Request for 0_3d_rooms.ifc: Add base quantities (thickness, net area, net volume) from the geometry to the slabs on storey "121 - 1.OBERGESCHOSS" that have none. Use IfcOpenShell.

First a look at what the model holds.

```python
import ifcopenshell
import ifcopenshell.util.element
import ifcopenshell.util.unit

model = ifcopenshell.open("0_3d_rooms.ifc")
print(model.schema)
for unit_type in ("LENGTHUNIT", "AREAUNIT", "VOLUMEUNIT"):
    print(unit_type, ifcopenshell.util.unit.calculate_unit_scale(model, unit_type))
storey = next(s for s in model.by_type("IfcBuildingStorey") if s.Name == "121 - 1.OBERGESCHOSS")
slabs = [e for e in ifcopenshell.util.element.get_decomposition(storey) if e.is_a("IfcSlab")]
for e in sorted(slabs, key=lambda e: e.id()):
    print(e.id(), e.is_a(), e.Name, list(ifcopenshell.util.element.get_psets(e, qtos_only=True)), sep=" | ")
```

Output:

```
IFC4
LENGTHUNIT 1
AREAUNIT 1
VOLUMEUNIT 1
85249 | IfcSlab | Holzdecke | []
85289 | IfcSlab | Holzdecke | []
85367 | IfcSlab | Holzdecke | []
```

```python
import ifcopenshell
import ifcopenshell.api.pset
import ifcopenshell.geom
import ifcopenshell.util.element
import ifcopenshell.util.shape
import ifcopenshell.util.unit

model = ifcopenshell.open("0_3d_rooms.ifc")
unit_scale = ifcopenshell.util.unit.calculate_unit_scale(model)
area_scale = ifcopenshell.util.unit.calculate_unit_scale(model, "AREAUNIT")
volume_scale = ifcopenshell.util.unit.calculate_unit_scale(model, "VOLUMEUNIT")
settings = ifcopenshell.geom.settings()

storey = next(s for s in model.by_type("IfcBuildingStorey") if s.Name == "121 - 1.OBERGESCHOSS")
slabs = [e for e in ifcopenshell.util.element.get_decomposition(storey) if e.is_a("IfcSlab")]

for e in sorted(slabs, key=lambda e: e.id()):
    if ifcopenshell.util.element.get_psets(e, qtos_only=True, should_inherit=False):
        continue
    # Geometry comes back in metres, in the element's own axes.
    shape = ifcopenshell.geom.create_shape(settings, e)
    values = {
        "Width": ifcopenshell.util.shape.get_z(shape.geometry) / unit_scale,
        "NetArea": ifcopenshell.util.shape.get_footprint_area(shape.geometry) / area_scale,
        "NetVolume": ifcopenshell.util.shape.get_volume(shape.geometry) / volume_scale,
    }
    qto = ifcopenshell.api.pset.add_qto(model, product=e, name="Qto_SlabBaseQuantities")
    ifcopenshell.api.pset.edit_qto(model, qto=qto, properties=values)
    print(e.id(), {k: round(v, 3) for k, v in values.items()})

model.write("0_3d_rooms-out.ifc")
```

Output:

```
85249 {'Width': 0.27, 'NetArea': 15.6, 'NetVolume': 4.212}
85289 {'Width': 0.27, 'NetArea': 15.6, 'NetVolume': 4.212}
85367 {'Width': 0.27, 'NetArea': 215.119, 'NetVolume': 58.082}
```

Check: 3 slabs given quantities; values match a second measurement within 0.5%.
